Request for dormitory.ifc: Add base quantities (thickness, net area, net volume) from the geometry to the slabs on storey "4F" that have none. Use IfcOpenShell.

First a look at what the model holds.

```python
import ifcopenshell
import ifcopenshell.util.element
import ifcopenshell.util.unit

model = ifcopenshell.open("dormitory.ifc")
print(model.schema)
for unit_type in ("LENGTHUNIT", "AREAUNIT", "VOLUMEUNIT"):
    print(unit_type, ifcopenshell.util.unit.calculate_unit_scale(model, unit_type))
storey = next(s for s in model.by_type("IfcBuildingStorey") if s.Name == "4F")
slabs = [e for e in ifcopenshell.util.element.get_decomposition(storey) if e.is_a("IfcSlab")]
for e in sorted(slabs, key=lambda e: e.id()):
    print(e.id(), e.is_a(), e.Name, list(ifcopenshell.util.element.get_psets(e, qtos_only=True)), sep=" | ")
```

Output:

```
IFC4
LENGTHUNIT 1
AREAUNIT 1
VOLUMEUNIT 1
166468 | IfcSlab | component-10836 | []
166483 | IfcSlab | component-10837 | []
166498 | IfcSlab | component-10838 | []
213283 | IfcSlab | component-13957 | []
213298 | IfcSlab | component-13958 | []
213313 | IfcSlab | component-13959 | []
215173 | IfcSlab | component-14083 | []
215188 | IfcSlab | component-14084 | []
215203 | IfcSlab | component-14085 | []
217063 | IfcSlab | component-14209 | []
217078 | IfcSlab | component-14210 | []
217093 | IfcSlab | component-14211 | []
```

```python
import ifcopenshell
import ifcopenshell.api.pset
import ifcopenshell.geom
import ifcopenshell.util.element
import ifcopenshell.util.shape
import ifcopenshell.util.unit

model = ifcopenshell.open("dormitory.ifc")
unit_scale = ifcopenshell.util.unit.calculate_unit_scale(model)
area_scale = ifcopenshell.util.unit.calculate_unit_scale(model, "AREAUNIT")
volume_scale = ifcopenshell.util.unit.calculate_unit_scale(model, "VOLUMEUNIT")
settings = ifcopenshell.geom.settings()

storey = next(s for s in model.by_type("IfcBuildingStorey") if s.Name == "4F")
slabs = [e for e in ifcopenshell.util.element.get_decomposition(storey) if e.is_a("IfcSlab")]

for e in sorted(slabs, key=lambda e: e.id()):
    if ifcopenshell.util.element.get_psets(e, qtos_only=True, should_inherit=False):
        continue
    # Geometry comes back in metres, in the element's own axes.
    shape = ifcopenshell.geom.create_shape(settings, e)
    values = {
        "Width": ifcopenshell.util.shape.get_z(shape.geometry) / unit_scale,
        "NetArea": ifcopenshell.util.shape.get_footprint_area(shape.geometry) / area_scale,
        "NetVolume": ifcopenshell.util.shape.get_volume(shape.geometry) / volume_scale,
    }
    qto = ifcopenshell.api.pset.add_qto(model, product=e, name="Qto_SlabBaseQuantities")
    ifcopenshell.api.pset.edit_qto(model, qto=qto, properties=values)
    print(e.id(), {k: round(v, 3) for k, v in values.items()})

model.write("dormitory_edited.ifc")
```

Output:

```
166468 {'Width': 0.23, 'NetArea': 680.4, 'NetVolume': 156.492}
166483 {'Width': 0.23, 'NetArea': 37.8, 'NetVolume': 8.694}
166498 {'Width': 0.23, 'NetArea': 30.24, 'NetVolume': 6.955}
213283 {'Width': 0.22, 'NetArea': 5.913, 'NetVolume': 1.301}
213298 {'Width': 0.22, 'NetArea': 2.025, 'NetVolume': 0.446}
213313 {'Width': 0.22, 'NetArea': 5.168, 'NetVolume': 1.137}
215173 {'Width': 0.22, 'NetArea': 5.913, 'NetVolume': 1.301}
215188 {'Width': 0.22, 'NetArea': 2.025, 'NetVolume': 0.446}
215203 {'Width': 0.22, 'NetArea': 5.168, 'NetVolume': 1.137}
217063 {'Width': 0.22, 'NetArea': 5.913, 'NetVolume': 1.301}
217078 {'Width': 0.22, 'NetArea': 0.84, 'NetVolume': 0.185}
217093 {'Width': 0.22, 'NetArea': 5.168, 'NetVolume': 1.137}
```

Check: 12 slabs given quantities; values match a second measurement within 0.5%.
